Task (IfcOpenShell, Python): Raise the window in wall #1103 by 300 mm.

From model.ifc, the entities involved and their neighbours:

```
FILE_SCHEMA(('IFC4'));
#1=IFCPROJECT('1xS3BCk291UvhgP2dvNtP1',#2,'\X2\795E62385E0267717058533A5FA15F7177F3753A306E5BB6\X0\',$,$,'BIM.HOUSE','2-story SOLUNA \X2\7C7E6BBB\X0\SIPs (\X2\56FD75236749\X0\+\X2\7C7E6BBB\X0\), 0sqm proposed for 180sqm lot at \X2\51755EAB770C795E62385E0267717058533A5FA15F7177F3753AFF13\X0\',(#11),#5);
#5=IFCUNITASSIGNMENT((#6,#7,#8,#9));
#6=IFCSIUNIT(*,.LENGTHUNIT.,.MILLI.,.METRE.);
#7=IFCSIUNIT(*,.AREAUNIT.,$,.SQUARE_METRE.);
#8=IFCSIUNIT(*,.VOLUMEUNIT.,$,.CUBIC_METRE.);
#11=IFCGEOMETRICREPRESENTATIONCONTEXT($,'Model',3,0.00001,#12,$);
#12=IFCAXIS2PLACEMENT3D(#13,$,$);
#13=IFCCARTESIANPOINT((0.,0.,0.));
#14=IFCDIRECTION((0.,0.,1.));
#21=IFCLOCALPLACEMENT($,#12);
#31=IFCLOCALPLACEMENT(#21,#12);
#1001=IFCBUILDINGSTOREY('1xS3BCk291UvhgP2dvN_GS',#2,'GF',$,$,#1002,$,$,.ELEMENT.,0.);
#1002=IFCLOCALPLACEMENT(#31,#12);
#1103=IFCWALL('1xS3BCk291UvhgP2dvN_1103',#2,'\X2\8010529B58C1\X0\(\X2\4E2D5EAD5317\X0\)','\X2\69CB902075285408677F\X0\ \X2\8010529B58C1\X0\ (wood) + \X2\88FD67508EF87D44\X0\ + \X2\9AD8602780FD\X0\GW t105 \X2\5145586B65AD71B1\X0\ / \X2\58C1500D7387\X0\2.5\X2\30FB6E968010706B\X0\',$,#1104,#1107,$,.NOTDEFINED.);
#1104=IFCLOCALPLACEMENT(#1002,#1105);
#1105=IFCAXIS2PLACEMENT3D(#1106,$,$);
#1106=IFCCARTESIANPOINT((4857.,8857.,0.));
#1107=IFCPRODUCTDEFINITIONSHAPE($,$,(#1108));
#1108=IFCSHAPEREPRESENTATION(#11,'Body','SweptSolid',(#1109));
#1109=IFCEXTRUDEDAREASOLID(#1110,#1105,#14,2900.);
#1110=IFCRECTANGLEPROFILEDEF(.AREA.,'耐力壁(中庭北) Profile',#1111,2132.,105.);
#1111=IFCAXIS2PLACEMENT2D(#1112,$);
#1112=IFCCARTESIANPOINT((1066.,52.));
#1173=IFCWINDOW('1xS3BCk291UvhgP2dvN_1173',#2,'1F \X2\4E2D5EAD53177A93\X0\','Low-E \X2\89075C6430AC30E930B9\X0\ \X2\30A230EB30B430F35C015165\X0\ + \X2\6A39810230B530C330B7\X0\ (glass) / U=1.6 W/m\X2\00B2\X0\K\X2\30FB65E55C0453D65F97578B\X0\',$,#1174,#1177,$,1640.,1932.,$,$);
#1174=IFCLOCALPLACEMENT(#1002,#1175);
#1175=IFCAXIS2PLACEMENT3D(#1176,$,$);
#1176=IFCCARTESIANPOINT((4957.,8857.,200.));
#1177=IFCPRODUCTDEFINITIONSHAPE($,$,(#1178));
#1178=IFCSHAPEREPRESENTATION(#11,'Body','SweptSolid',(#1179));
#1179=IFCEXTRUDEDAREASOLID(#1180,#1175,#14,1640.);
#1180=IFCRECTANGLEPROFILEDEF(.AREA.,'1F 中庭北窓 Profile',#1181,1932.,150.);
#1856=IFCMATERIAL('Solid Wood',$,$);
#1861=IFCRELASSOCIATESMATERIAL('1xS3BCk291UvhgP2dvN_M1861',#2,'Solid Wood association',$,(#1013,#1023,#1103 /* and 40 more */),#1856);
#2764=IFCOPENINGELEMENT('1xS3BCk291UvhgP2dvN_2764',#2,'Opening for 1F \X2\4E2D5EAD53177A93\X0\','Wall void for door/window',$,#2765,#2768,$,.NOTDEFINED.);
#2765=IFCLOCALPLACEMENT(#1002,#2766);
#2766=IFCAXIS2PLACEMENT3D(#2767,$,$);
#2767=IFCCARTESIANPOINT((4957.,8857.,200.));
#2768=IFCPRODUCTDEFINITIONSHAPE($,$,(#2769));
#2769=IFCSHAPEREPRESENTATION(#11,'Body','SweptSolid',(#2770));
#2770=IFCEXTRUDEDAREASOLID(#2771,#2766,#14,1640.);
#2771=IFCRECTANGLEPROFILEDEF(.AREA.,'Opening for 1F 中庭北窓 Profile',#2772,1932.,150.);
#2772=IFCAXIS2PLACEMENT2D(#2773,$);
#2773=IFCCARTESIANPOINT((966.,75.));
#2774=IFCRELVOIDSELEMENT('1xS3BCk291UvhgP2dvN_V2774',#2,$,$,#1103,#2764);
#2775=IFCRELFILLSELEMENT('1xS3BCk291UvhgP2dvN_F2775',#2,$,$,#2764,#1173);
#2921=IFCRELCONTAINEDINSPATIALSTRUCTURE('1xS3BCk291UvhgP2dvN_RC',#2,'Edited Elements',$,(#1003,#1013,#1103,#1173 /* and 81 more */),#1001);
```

```python
import numpy as np
import ifcopenshell
import ifcopenshell.api.geometry
import ifcopenshell.util.placement
import ifcopenshell.util.unit

model = ifcopenshell.open("model.ifc")
unit_scale = ifcopenshell.util.unit.calculate_unit_scale(model)

window = model.by_guid("1xS3BCk291UvhgP2dvN_1173")
opening = window.FillsVoids[0].RelatingOpeningElement
dz = 0.3 / unit_scale

shift = np.array([0.0, 0.0, dz])
# The window is not placed relative to its opening, so move both.
for product in (opening, window):
    matrix = ifcopenshell.util.placement.get_local_placement(product.ObjectPlacement)
    matrix[:3, 3] += shift
    ifcopenshell.api.geometry.edit_object_placement(model, product=product, matrix=matrix, is_si=False)

print(f"moved by {dz * unit_scale:+.3f} m")

model.write("model_updated.ifc")
```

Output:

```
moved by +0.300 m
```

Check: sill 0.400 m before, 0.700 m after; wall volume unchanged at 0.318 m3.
